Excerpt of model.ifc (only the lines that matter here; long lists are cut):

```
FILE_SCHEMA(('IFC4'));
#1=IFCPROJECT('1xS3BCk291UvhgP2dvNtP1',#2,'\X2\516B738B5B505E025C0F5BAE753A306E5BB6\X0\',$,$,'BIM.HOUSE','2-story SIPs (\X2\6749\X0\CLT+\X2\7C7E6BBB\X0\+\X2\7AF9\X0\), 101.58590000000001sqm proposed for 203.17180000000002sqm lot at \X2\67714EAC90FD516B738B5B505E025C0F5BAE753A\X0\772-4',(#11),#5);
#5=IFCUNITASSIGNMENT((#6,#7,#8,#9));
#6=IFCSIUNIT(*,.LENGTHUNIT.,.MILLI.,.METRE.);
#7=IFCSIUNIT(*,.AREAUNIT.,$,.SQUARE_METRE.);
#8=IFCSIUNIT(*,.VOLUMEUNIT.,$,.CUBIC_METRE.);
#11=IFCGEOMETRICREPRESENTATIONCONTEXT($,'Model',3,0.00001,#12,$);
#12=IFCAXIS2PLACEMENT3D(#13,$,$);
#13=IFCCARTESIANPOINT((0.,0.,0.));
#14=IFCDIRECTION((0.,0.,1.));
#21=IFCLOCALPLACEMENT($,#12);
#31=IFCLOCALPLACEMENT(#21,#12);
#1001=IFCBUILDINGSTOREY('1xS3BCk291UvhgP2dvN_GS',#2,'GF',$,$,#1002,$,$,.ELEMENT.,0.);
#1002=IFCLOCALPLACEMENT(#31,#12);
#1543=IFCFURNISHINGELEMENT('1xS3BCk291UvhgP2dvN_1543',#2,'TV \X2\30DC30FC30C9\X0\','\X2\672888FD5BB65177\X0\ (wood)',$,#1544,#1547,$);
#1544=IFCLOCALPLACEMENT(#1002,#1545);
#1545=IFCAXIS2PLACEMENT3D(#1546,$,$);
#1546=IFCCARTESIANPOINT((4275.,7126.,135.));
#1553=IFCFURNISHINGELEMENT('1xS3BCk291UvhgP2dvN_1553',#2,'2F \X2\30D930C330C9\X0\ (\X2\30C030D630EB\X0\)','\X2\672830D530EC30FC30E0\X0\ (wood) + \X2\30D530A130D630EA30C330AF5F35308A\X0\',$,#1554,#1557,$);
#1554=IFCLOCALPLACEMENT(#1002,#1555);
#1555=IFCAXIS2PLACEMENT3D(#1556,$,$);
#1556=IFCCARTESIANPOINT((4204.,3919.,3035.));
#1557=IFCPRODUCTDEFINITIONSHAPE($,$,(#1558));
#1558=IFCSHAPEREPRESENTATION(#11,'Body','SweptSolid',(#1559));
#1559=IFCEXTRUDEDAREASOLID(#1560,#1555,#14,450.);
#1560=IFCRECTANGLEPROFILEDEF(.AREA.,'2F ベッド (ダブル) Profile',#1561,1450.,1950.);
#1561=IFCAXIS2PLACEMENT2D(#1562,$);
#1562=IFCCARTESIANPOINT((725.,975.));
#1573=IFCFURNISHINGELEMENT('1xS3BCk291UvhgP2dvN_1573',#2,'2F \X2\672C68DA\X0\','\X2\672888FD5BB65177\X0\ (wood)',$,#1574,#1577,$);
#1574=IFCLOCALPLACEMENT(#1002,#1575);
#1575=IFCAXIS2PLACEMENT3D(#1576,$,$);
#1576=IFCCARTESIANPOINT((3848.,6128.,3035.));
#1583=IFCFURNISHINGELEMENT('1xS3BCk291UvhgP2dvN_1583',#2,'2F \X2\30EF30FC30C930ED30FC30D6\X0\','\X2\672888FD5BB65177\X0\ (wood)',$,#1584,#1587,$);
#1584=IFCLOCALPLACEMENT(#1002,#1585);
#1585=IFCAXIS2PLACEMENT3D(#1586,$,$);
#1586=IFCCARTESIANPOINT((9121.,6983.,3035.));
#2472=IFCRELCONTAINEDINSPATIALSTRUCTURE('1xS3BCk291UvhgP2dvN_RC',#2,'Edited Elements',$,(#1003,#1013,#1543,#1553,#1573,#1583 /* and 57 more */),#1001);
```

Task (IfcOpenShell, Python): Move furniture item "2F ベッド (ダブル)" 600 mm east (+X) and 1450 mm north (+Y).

```python
import ifcopenshell
import ifcopenshell.api.geometry
import ifcopenshell.util.placement
import ifcopenshell.util.unit

model = ifcopenshell.open("model.ifc")
unit_scale = ifcopenshell.util.unit.calculate_unit_scale(model)

item = model.by_guid("1xS3BCk291UvhgP2dvN_1553")
matrix = ifcopenshell.util.placement.get_local_placement(item.ObjectPlacement)
matrix[0, 3] += 0.6 / unit_scale
matrix[1, 3] += 1.45 / unit_scale
ifcopenshell.api.geometry.edit_object_placement(model, product=item, matrix=matrix, is_si=False)

print(ifcopenshell.util.placement.get_local_placement(item.ObjectPlacement).round(3) + 0.0)

model.write("model_v2.ifc")
```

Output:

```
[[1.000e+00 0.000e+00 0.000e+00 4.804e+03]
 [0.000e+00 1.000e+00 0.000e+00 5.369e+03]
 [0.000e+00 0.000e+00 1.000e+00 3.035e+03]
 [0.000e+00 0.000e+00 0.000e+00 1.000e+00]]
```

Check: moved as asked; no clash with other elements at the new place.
